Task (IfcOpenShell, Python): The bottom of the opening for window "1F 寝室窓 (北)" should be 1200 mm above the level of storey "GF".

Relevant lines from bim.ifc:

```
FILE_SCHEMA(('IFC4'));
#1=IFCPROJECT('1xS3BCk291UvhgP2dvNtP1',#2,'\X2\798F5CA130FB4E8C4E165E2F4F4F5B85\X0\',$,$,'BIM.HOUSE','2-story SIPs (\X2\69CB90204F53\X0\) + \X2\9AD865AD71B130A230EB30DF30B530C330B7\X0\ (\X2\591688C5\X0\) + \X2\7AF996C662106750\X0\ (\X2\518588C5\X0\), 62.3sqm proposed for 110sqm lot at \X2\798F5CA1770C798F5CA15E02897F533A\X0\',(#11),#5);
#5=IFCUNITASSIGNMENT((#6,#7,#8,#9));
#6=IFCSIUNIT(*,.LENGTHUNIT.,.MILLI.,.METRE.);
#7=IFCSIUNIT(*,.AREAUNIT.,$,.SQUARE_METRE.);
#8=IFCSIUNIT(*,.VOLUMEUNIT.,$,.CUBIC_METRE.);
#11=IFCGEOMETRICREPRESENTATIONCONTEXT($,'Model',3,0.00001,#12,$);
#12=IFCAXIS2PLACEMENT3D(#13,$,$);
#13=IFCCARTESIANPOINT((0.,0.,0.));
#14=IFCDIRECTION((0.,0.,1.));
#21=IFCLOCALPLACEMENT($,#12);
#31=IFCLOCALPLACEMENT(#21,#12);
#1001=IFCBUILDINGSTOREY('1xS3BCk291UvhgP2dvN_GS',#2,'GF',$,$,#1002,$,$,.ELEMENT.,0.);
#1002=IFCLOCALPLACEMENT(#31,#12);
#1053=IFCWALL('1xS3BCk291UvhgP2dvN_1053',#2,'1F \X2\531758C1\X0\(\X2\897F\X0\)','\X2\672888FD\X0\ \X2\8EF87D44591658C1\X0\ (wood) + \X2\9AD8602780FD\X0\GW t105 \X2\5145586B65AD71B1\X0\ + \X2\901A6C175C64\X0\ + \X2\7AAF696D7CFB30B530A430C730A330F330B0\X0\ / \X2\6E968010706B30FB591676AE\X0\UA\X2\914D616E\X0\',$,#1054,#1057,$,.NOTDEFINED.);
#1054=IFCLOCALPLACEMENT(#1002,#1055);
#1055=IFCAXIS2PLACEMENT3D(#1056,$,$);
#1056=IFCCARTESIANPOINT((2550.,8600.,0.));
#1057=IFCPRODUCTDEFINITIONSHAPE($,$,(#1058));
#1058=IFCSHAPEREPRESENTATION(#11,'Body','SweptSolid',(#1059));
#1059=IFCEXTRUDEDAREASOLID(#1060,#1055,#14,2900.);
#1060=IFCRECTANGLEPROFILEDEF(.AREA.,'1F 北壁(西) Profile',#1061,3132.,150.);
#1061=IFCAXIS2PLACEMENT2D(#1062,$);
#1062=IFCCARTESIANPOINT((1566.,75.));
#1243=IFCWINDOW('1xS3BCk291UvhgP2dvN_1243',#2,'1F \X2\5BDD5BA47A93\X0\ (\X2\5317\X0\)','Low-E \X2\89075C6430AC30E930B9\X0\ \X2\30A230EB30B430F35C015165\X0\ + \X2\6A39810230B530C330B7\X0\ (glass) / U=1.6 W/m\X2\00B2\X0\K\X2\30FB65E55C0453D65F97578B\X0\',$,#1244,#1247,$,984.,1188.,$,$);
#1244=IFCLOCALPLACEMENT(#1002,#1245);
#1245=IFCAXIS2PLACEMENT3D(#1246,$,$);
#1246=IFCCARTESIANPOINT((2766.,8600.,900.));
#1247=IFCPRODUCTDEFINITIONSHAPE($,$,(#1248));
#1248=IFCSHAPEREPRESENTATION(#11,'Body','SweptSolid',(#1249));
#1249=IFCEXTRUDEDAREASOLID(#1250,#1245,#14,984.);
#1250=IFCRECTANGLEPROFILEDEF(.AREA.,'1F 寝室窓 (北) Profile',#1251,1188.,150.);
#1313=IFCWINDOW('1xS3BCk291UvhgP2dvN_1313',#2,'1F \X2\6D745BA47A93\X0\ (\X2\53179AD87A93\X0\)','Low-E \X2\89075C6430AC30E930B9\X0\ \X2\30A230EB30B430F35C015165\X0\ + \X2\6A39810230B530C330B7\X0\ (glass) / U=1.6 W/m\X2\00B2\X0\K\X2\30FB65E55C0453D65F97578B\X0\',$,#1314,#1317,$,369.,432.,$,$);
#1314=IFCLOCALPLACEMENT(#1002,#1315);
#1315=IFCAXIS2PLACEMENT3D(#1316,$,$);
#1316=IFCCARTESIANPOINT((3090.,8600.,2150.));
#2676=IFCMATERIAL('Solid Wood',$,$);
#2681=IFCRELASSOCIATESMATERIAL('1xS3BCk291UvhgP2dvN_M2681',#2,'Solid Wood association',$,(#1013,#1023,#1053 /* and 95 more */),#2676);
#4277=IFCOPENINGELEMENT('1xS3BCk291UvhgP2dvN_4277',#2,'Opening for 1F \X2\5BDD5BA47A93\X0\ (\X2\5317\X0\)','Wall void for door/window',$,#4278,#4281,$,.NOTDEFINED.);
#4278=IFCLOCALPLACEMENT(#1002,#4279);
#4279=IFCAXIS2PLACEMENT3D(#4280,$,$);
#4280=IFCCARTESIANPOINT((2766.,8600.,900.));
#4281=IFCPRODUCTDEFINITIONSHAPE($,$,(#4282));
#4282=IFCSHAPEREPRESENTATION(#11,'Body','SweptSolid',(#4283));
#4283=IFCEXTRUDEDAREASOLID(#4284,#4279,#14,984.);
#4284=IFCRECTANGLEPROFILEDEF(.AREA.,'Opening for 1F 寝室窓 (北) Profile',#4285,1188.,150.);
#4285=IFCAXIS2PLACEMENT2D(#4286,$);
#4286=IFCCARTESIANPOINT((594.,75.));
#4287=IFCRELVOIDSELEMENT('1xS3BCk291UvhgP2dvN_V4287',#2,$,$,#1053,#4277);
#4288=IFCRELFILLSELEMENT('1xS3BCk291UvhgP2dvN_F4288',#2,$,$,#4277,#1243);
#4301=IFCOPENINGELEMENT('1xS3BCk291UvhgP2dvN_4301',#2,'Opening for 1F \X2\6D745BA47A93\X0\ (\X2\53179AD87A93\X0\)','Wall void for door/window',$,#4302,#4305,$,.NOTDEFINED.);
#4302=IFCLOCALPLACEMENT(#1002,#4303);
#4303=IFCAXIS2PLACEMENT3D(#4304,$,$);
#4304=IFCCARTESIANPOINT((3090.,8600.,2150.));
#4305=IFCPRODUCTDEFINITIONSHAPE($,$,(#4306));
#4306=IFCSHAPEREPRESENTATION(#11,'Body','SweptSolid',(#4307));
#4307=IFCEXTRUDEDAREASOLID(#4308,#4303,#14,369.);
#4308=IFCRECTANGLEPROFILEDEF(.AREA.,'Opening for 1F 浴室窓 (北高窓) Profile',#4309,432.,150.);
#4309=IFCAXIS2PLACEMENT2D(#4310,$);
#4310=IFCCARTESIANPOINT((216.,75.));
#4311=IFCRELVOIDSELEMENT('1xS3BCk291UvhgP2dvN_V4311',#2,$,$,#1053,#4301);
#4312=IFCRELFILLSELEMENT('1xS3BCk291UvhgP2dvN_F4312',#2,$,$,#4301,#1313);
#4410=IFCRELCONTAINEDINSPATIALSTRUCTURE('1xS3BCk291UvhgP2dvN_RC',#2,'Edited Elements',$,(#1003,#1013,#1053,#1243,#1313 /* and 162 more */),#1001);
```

```python
import numpy as np
import ifcopenshell
import ifcopenshell.api.geometry
import ifcopenshell.geom
import ifcopenshell.util.element
import ifcopenshell.util.placement
import ifcopenshell.util.shape
import ifcopenshell.util.unit

model = ifcopenshell.open("bim.ifc")
unit_scale = ifcopenshell.util.unit.calculate_unit_scale(model)

window = model.by_guid("1xS3BCk291UvhgP2dvN_1243")
opening = window.FillsVoids[0].RelatingOpeningElement
storey = ifcopenshell.util.element.get_container(window, ifc_class="IfcBuildingStorey")
level = ifcopenshell.util.placement.get_local_placement(storey.ObjectPlacement)[2, 3]

# The opening's origin need not be at the sill, so measure its lowest point.
shape = ifcopenshell.geom.create_shape(ifcopenshell.geom.settings(), opening)
bottom = ifcopenshell.util.shape.get_shape_bottom_elevation(shape, shape.geometry) / unit_scale
dz = level + 1.2 / unit_scale - bottom

shift = np.array([0.0, 0.0, dz])
# The window is not placed relative to its opening, so move both.
for product in (opening, window):
    matrix = ifcopenshell.util.placement.get_local_placement(product.ObjectPlacement)
    matrix[:3, 3] += shift
    ifcopenshell.api.geometry.edit_object_placement(model, product=product, matrix=matrix, is_si=False)

print(f"moved by {dz * unit_scale:+.3f} m")

model.write("bim_rev.ifc")
```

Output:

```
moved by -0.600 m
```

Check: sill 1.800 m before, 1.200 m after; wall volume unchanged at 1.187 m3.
